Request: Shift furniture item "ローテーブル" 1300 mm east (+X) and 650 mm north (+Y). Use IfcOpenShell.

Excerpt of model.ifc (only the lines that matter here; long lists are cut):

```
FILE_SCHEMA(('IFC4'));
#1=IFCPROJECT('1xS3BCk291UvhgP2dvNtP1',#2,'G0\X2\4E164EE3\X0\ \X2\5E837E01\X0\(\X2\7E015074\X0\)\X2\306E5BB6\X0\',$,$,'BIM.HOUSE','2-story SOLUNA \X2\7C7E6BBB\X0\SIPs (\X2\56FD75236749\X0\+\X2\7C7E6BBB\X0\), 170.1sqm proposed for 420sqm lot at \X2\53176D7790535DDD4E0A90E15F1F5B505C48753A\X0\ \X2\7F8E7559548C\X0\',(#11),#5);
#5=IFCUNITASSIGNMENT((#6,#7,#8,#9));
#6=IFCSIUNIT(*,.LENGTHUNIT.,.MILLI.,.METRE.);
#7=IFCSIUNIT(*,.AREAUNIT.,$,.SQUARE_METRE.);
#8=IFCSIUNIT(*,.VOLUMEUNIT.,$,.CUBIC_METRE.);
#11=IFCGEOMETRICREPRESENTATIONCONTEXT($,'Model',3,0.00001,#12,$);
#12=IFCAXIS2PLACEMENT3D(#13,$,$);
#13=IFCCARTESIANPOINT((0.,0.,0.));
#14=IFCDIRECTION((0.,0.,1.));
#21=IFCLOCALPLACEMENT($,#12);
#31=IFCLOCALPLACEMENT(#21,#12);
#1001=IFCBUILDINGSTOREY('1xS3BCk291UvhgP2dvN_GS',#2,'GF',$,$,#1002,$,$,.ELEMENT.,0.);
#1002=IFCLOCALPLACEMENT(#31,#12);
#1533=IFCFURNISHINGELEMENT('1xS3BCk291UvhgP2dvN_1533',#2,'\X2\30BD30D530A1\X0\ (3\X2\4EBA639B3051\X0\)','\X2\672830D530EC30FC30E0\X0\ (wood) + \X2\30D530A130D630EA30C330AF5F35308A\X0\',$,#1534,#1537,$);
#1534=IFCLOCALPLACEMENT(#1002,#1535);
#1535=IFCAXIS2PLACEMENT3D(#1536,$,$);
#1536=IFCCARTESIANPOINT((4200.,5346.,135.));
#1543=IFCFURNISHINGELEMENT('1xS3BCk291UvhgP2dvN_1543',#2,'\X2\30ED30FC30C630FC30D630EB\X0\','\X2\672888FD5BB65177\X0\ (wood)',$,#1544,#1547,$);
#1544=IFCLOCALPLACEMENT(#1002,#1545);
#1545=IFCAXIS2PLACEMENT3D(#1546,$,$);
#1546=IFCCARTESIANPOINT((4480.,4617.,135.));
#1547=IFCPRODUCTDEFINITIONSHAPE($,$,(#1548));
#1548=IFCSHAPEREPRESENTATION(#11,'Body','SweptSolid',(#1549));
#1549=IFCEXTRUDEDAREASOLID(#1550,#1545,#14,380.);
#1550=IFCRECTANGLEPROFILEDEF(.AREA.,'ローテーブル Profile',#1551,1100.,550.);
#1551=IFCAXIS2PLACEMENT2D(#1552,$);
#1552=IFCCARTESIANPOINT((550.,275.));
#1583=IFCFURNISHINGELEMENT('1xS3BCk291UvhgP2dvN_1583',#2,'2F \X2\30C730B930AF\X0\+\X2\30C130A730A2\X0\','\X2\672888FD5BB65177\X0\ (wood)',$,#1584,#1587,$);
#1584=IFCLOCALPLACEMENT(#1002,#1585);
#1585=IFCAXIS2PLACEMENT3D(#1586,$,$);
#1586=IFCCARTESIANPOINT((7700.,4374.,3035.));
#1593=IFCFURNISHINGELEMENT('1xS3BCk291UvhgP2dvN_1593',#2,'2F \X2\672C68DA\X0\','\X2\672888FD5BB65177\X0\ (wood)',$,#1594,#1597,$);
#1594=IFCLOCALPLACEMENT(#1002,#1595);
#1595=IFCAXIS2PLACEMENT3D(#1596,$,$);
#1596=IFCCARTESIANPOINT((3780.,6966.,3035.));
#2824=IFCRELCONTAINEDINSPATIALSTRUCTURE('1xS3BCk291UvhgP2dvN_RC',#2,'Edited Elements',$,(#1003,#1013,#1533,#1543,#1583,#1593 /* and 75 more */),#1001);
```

```python
import ifcopenshell
import ifcopenshell.api.geometry
import ifcopenshell.util.placement

model = ifcopenshell.open("model.ifc")

item = model.by_id(1543)
matrix = ifcopenshell.util.placement.get_local_placement(item.ObjectPlacement)
matrix[0, 3] += 1300.0
matrix[1, 3] += 650.0
ifcopenshell.api.geometry.edit_object_placement(model, product=item, matrix=matrix, is_si=False)

print(ifcopenshell.util.placement.get_local_placement(item.ObjectPlacement).round(3) + 0.0)

model.write("model_rev.ifc")
```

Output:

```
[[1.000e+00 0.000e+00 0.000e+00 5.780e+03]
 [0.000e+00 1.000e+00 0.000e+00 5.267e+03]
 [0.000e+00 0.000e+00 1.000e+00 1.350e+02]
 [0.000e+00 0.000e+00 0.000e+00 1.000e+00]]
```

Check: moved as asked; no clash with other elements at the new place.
